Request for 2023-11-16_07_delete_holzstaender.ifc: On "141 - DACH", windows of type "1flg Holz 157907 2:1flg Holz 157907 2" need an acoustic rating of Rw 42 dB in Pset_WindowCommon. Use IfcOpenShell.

First a look at what the model holds.

```python
import ifcopenshell
import ifcopenshell.util.element

model = ifcopenshell.open("2023-11-16_07_delete_holzstaender.ifc")
print(model.schema)
storey = next(s for s in model.by_type("IfcBuildingStorey") if s.Name == "141 - DACH")
windows = [e for e in ifcopenshell.util.element.get_decomposition(storey) if e.is_a("IfcWindow")]
seen = {}
for e in windows:
    element_type = ifcopenshell.util.element.get_type(e)
    key = (element_type.Name if element_type != e and element_type else None, ifcopenshell.util.element.get_pset(e, "Pset_WindowCommon", "AcousticRating"))
    seen[key] = seen.get(key, 0) + 1
for (name, value), count in sorted(seen.items(), key=str):
    print(count, "x", name, "|", value)
```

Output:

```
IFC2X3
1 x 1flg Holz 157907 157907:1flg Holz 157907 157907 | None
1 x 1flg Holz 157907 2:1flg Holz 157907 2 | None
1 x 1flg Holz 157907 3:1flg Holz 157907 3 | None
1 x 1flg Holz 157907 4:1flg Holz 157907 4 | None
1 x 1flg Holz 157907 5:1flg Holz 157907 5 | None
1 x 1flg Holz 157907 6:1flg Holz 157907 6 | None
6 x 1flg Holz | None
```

```python
import ifcopenshell
import ifcopenshell.api.pset
import ifcopenshell.util.element

model = ifcopenshell.open("2023-11-16_07_delete_holzstaender.ifc")

storey = next(s for s in model.by_type("IfcBuildingStorey") if s.Name == "141 - DACH")
windows = [e for e in ifcopenshell.util.element.get_decomposition(storey) if e.is_a("IfcWindow")]

count = 0
for e in windows:
    element_type = ifcopenshell.util.element.get_type(e)
    if element_type in (None, e) or element_type.Name != "1flg Holz 157907 2:1flg Holz 157907 2":
        continue
    # add_pset returns the element's existing set when there is one.
    pset = ifcopenshell.api.pset.add_pset(model, product=e, name="Pset_WindowCommon")
    ifcopenshell.api.pset.edit_pset(model, pset=pset, properties={"AcousticRating": "Rw 42 dB"})
    count += 1

print(count, "windows updated")

model.write("2023-11-16_07_delete_holzstaender-out.ifc")
```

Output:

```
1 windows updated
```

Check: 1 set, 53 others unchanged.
